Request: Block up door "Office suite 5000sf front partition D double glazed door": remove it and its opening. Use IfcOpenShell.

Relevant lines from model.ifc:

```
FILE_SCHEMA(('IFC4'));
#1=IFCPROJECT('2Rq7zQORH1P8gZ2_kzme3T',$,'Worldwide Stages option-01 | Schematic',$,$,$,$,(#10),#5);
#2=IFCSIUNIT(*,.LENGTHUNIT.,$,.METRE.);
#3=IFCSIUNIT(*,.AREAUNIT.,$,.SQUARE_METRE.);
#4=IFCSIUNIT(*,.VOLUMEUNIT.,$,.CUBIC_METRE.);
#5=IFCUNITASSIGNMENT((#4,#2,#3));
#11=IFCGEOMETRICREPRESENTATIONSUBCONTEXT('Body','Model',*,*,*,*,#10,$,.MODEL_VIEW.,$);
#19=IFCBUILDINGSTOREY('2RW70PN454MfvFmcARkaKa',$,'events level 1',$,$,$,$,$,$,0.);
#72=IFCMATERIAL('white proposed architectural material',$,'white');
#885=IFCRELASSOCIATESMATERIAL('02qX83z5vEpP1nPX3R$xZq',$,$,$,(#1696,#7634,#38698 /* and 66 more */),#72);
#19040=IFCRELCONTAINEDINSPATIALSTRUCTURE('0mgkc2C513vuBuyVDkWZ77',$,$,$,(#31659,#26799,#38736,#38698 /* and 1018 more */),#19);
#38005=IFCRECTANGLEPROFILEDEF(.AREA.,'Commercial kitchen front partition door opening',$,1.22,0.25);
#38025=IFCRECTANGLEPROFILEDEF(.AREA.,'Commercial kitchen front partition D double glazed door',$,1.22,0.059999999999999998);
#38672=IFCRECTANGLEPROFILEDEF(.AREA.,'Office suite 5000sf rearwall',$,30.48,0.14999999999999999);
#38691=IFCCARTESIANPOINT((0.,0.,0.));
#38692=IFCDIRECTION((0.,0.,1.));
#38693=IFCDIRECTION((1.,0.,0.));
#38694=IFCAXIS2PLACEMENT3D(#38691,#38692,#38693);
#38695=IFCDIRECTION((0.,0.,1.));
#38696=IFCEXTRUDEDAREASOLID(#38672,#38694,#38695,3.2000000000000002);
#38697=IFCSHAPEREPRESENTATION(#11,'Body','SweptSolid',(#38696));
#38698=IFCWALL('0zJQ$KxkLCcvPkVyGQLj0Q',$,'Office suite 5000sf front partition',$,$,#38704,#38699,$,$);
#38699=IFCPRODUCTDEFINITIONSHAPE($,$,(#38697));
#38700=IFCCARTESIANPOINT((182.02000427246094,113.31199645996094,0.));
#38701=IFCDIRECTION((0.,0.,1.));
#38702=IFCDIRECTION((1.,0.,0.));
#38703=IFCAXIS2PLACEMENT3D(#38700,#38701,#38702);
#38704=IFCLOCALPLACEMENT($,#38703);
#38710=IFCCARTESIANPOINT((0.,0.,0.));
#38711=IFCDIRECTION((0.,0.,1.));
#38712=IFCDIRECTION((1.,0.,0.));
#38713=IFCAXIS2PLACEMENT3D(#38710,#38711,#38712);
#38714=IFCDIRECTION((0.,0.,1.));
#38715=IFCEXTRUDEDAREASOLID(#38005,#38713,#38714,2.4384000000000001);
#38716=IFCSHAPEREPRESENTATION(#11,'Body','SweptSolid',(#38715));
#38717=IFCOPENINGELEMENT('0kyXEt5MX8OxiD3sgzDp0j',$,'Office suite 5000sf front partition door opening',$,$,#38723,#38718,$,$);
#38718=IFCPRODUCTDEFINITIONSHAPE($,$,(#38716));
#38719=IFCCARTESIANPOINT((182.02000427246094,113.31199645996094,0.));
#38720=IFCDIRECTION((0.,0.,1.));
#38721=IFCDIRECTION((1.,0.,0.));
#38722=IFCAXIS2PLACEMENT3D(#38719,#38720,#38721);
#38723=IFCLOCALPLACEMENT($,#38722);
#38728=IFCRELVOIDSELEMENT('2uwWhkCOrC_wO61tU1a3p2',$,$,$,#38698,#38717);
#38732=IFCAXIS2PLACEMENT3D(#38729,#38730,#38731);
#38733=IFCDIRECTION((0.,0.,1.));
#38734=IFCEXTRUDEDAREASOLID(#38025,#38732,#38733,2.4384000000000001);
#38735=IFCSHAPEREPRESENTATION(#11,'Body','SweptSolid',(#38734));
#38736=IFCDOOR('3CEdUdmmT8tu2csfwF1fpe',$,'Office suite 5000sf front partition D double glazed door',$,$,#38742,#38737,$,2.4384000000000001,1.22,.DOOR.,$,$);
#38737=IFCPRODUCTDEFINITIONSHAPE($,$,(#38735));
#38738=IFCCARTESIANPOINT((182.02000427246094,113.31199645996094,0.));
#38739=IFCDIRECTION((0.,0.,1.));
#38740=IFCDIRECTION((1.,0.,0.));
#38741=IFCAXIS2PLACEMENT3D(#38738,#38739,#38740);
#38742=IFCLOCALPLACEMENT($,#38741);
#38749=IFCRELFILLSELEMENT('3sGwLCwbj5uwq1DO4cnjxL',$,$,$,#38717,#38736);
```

```python
import ifcopenshell
import ifcopenshell.api.feature
import ifcopenshell.api.root
import ifcopenshell.geom
import ifcopenshell.util.shape

model = ifcopenshell.open("model.ifc")
settings = ifcopenshell.geom.settings()


def volume(element):
    """Net volume in cubic metres, openings subtracted."""
    shape = ifcopenshell.geom.create_shape(settings, element)
    return ifcopenshell.util.shape.get_volume(shape.geometry)


door = model.by_guid("3CEdUdmmT8tu2csfwF1fpe")
opening = door.FillsVoids[0].RelatingOpeningElement
wall = opening.VoidsElements[0].RelatingBuildingElement
before = volume(wall)

ifcopenshell.api.root.remove_product(model, product=door)
ifcopenshell.api.feature.remove_feature(model, feature=opening)

after = volume(wall)

print(f"wall volume {before:.3f} -> {after:.3f} m3")

model.write("model_v2.ifc")
```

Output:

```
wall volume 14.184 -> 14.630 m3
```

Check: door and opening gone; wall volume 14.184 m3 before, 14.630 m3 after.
